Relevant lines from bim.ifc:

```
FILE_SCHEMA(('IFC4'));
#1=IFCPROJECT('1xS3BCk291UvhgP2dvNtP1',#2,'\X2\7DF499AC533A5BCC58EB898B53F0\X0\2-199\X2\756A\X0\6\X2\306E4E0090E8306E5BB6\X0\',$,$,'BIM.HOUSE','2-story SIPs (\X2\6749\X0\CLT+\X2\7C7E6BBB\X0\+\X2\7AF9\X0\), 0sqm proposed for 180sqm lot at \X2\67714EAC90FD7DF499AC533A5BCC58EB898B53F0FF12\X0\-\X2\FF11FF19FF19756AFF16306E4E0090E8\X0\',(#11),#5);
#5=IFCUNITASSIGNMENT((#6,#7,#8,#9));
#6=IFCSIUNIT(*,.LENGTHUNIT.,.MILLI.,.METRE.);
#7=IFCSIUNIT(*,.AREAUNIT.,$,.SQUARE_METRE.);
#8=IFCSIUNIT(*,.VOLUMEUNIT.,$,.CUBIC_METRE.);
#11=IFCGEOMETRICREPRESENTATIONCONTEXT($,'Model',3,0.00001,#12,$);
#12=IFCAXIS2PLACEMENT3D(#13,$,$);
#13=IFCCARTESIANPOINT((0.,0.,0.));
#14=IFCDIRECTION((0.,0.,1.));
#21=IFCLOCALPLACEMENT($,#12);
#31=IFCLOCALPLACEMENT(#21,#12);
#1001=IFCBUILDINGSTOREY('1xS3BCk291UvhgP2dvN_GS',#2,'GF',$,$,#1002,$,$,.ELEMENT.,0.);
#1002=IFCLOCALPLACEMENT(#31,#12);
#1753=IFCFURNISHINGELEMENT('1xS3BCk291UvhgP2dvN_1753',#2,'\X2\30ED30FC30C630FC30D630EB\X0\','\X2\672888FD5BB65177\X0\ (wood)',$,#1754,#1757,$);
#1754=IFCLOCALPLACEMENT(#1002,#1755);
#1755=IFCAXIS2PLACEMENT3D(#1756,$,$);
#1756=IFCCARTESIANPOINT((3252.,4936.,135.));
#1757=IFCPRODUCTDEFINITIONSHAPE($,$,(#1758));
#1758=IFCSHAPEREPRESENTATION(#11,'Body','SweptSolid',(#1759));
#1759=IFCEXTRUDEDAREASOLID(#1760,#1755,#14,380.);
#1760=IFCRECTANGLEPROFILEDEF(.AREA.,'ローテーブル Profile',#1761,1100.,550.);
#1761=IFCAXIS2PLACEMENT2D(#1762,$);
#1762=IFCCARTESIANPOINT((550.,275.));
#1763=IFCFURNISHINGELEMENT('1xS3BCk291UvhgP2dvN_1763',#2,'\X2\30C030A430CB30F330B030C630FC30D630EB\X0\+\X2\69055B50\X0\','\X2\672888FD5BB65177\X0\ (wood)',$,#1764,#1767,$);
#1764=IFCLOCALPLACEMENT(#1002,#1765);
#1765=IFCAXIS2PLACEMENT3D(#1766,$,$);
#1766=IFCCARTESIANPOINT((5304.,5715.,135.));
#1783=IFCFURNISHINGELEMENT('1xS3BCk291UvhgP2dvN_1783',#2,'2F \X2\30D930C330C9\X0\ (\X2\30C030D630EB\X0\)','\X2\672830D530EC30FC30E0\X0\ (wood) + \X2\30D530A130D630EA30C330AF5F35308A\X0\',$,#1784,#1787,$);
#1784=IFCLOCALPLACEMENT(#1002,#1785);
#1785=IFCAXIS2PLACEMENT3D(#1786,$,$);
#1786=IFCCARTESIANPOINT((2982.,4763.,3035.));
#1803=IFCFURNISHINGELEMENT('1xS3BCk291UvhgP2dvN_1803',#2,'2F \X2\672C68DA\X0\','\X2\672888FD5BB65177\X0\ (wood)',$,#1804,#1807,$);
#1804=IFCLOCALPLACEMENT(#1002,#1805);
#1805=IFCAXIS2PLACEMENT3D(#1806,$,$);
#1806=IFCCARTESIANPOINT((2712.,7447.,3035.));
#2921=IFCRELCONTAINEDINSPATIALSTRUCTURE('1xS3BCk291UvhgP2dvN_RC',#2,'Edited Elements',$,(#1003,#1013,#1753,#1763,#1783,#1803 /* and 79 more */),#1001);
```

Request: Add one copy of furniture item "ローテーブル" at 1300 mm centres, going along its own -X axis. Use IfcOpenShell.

```python
import ifcopenshell
import ifcopenshell.api.geometry
import ifcopenshell.api.root
import ifcopenshell.util.element
import ifcopenshell.util.placement
import ifcopenshell.util.unit

model = ifcopenshell.open("bim.ifc")
unit_scale = ifcopenshell.util.unit.calculate_unit_scale(model)


def reuse_history(source, copy):
    """copy_class also copies each property set's owner history, people and application; keep the originals."""
    for rel in copy.IsDefinedBy:
        if rel.is_a("IfcRelDefinesByProperties") and (history := rel.RelatingPropertyDefinition.OwnerHistory):
            rel.RelatingPropertyDefinition.OwnerHistory = source.OwnerHistory
            ifcopenshell.util.element.remove_deep2(model, history)


source = model.by_guid("1xS3BCk291UvhgP2dvN_1753")
base = ifcopenshell.util.placement.get_local_placement(source.ObjectPlacement)
step = -base[:3, 0] * 1.3 / unit_scale

for i in range(1, 2):
    copy = ifcopenshell.api.root.copy_class(model, product=source)
    copy.Representation = ifcopenshell.util.element.copy_deep(
        model, source.Representation, exclude=["IfcGeometricRepresentationContext", "IfcRepresentationMap"]
    )
    reuse_history(source, copy)
    matrix = base.copy()
    matrix[:3, 3] += i * step
    print("added at", matrix[:3, 3].round(3) + 0.0)
    ifcopenshell.api.geometry.edit_object_placement(model, product=copy, matrix=matrix, is_si=False)

model.write("bim_rev.ifc")
```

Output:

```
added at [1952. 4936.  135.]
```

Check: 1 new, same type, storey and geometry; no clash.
